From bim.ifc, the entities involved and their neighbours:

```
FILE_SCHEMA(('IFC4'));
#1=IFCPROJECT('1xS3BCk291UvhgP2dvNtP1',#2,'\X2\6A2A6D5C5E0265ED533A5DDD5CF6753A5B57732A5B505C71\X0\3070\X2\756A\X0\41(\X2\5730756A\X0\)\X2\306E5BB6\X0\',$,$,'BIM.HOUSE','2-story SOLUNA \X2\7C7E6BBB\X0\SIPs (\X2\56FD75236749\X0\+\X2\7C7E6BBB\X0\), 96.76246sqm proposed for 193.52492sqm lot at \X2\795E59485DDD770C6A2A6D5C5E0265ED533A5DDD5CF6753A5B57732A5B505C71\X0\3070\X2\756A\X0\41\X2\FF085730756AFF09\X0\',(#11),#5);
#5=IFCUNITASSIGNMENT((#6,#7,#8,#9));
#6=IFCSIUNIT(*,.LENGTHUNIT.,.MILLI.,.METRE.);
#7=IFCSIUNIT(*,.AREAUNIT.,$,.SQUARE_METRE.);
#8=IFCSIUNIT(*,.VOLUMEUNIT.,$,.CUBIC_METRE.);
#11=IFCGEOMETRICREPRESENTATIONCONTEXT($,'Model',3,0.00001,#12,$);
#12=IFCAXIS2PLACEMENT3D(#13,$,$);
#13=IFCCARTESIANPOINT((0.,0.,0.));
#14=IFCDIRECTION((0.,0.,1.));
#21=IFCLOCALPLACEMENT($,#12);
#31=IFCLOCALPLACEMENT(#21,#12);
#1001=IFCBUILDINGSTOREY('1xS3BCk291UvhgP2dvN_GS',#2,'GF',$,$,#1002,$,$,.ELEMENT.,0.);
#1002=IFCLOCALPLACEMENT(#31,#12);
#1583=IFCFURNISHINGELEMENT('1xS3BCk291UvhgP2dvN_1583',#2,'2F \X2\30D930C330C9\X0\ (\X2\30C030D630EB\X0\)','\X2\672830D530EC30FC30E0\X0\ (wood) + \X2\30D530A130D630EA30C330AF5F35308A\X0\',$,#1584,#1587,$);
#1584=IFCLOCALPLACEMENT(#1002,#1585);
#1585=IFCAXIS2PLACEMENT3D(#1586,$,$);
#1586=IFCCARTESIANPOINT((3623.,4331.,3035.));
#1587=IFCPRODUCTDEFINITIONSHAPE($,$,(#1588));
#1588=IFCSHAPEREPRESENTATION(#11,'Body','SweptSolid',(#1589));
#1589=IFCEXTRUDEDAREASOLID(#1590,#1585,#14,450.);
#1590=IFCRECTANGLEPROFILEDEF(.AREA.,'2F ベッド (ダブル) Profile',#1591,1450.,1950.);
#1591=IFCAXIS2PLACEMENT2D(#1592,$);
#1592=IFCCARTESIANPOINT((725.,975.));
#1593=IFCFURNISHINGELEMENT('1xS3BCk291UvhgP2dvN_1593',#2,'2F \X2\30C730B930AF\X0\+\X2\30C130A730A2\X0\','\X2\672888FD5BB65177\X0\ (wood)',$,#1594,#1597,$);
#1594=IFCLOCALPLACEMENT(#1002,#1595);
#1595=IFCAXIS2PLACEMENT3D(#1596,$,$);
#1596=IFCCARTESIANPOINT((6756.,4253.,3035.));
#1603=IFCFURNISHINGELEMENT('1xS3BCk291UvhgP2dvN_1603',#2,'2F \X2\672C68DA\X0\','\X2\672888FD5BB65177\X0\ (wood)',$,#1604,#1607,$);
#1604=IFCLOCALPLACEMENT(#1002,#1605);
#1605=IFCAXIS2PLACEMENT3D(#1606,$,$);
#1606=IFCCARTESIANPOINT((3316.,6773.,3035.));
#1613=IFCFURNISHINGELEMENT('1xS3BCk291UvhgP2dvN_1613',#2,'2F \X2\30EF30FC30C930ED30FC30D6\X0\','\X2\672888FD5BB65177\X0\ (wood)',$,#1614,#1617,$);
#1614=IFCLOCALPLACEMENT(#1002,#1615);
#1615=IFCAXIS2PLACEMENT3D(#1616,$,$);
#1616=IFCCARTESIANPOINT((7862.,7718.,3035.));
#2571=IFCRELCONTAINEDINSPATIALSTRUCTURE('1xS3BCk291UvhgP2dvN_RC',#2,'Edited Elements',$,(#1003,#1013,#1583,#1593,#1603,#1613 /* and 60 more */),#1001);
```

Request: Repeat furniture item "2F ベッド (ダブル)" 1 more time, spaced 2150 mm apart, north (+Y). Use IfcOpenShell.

```python
import numpy as np
import ifcopenshell
import ifcopenshell.api.geometry
import ifcopenshell.api.root
import ifcopenshell.util.element
import ifcopenshell.util.placement
import ifcopenshell.util.unit

model = ifcopenshell.open("bim.ifc")
unit_scale = ifcopenshell.util.unit.calculate_unit_scale(model)


def reuse_history(source, copy):
    """copy_class also copies each property set's owner history, people and application; keep the originals."""
    for rel in copy.IsDefinedBy:
        if rel.is_a("IfcRelDefinesByProperties") and (history := rel.RelatingPropertyDefinition.OwnerHistory):
            rel.RelatingPropertyDefinition.OwnerHistory = source.OwnerHistory
            ifcopenshell.util.element.remove_deep2(model, history)


source = model.by_guid("1xS3BCk291UvhgP2dvN_1583")
base = ifcopenshell.util.placement.get_local_placement(source.ObjectPlacement)
step = np.array([0.0, 1.0, 0.0]) * 2.15 / unit_scale

for i in range(1, 2):
    copy = ifcopenshell.api.root.copy_class(model, product=source)
    copy.Representation = ifcopenshell.util.element.copy_deep(
        model, source.Representation, exclude=["IfcGeometricRepresentationContext", "IfcRepresentationMap"]
    )
    reuse_history(source, copy)
    matrix = base.copy()
    matrix[:3, 3] += i * step
    print("added at", matrix[:3, 3].round(3) + 0.0)
    ifcopenshell.api.geometry.edit_object_placement(model, product=copy, matrix=matrix, is_si=False)

model.write("bim_updated.ifc")
```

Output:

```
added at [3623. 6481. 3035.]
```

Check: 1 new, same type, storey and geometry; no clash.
